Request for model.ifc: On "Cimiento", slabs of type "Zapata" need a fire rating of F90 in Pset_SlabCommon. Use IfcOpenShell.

First a look at what the model holds.

```python
import ifcopenshell
import ifcopenshell.util.element

model = ifcopenshell.open("model.ifc")
print(model.schema)
storey = next(s for s in model.by_type("IfcBuildingStorey") if s.Name == "Cimiento")
slabs = [e for e in ifcopenshell.util.element.get_decomposition(storey) if e.is_a("IfcSlab")]
seen = {}
for e in slabs:
    element_type = ifcopenshell.util.element.get_type(e)
    key = (element_type.Name if element_type != e and element_type else None, ifcopenshell.util.element.get_pset(e, "Pset_SlabCommon", "FireRating"))
    seen[key] = seen.get(key, 0) + 1
for (name, value), count in sorted(seen.items(), key=str):
    print(count, "x", name, "|", value)
```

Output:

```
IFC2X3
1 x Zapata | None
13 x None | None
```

```python
import ifcopenshell
import ifcopenshell.api.pset
import ifcopenshell.util.element

model = ifcopenshell.open("model.ifc")

storey = next(s for s in model.by_type("IfcBuildingStorey") if s.Name == "Cimiento")
slabs = [e for e in ifcopenshell.util.element.get_decomposition(storey) if e.is_a("IfcSlab")]

count = 0
for e in slabs:
    element_type = ifcopenshell.util.element.get_type(e)
    if element_type in (None, e) or element_type.Name != "Zapata":
        continue
    # add_pset returns the element's existing set when there is one.
    pset = ifcopenshell.api.pset.add_pset(model, product=e, name="Pset_SlabCommon")
    ifcopenshell.api.pset.edit_pset(model, pset=pset, properties={"FireRating": "F90"})
    count += 1

print(count, "slabs updated")

model.write("model_rev.ifc")
```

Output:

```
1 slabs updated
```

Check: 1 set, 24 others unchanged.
